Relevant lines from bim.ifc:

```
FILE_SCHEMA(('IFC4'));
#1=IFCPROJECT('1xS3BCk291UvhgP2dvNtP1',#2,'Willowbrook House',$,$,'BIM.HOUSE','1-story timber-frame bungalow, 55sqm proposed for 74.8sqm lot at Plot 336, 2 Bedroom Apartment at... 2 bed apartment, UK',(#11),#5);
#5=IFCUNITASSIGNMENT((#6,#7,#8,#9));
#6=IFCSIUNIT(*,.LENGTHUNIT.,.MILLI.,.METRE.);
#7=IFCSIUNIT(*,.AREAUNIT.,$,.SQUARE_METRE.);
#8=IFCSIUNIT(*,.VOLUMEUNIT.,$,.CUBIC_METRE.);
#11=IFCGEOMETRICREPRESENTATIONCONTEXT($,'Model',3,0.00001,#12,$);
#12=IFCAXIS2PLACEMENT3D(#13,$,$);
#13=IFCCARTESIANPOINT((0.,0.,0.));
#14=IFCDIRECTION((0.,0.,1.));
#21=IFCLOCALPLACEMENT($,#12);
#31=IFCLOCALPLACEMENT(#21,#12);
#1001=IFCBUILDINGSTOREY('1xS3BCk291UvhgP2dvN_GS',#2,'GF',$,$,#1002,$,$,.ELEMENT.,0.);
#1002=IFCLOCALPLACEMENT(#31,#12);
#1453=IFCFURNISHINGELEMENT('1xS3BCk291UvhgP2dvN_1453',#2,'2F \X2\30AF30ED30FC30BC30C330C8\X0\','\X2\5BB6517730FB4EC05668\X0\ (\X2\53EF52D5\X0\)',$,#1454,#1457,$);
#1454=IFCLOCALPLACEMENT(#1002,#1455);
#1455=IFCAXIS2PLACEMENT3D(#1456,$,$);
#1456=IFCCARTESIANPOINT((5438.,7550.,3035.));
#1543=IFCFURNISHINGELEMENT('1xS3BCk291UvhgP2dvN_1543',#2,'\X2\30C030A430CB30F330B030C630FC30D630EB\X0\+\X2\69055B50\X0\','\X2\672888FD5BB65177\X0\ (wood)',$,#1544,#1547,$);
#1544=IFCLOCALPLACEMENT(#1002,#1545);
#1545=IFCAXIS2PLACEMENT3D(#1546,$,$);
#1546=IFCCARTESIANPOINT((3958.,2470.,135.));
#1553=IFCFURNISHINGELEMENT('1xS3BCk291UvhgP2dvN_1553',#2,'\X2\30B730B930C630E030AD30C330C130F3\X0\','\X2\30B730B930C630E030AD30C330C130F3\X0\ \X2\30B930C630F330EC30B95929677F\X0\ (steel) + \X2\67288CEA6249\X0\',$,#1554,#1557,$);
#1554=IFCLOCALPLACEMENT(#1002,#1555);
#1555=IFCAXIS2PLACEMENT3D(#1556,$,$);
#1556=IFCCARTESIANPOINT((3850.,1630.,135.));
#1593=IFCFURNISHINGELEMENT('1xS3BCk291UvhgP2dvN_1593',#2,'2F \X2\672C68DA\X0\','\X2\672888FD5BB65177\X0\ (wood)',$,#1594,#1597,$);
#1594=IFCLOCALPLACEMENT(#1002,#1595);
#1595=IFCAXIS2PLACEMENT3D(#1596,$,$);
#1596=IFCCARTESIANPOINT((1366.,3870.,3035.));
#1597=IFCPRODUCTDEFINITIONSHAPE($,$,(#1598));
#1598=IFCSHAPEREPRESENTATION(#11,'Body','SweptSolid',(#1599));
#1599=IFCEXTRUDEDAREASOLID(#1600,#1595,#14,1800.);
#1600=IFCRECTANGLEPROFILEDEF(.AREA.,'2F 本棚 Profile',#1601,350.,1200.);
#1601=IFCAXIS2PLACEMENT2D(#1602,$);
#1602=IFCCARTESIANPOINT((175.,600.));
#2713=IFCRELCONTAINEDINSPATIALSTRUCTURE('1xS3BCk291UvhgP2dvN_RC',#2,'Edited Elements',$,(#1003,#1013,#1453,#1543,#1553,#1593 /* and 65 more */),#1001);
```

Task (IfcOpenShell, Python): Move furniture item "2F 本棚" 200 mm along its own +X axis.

```python
import ifcopenshell
import ifcopenshell.api.geometry
import ifcopenshell.util.placement

model = ifcopenshell.open("bim.ifc")

item = model.by_guid("1xS3BCk291UvhgP2dvN_1593")
matrix = ifcopenshell.util.placement.get_local_placement(item.ObjectPlacement)
matrix[:3, 3] += matrix[:3, 0] * 200.0
ifcopenshell.api.geometry.edit_object_placement(model, product=item, matrix=matrix, is_si=False)

print(ifcopenshell.util.placement.get_local_placement(item.ObjectPlacement).round(3) + 0.0)

model.write("bim_updated.ifc")
```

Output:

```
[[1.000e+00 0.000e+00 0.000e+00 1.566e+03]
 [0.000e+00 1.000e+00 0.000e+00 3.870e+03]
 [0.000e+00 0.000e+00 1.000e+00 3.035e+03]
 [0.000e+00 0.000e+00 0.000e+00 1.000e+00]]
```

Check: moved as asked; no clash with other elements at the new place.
